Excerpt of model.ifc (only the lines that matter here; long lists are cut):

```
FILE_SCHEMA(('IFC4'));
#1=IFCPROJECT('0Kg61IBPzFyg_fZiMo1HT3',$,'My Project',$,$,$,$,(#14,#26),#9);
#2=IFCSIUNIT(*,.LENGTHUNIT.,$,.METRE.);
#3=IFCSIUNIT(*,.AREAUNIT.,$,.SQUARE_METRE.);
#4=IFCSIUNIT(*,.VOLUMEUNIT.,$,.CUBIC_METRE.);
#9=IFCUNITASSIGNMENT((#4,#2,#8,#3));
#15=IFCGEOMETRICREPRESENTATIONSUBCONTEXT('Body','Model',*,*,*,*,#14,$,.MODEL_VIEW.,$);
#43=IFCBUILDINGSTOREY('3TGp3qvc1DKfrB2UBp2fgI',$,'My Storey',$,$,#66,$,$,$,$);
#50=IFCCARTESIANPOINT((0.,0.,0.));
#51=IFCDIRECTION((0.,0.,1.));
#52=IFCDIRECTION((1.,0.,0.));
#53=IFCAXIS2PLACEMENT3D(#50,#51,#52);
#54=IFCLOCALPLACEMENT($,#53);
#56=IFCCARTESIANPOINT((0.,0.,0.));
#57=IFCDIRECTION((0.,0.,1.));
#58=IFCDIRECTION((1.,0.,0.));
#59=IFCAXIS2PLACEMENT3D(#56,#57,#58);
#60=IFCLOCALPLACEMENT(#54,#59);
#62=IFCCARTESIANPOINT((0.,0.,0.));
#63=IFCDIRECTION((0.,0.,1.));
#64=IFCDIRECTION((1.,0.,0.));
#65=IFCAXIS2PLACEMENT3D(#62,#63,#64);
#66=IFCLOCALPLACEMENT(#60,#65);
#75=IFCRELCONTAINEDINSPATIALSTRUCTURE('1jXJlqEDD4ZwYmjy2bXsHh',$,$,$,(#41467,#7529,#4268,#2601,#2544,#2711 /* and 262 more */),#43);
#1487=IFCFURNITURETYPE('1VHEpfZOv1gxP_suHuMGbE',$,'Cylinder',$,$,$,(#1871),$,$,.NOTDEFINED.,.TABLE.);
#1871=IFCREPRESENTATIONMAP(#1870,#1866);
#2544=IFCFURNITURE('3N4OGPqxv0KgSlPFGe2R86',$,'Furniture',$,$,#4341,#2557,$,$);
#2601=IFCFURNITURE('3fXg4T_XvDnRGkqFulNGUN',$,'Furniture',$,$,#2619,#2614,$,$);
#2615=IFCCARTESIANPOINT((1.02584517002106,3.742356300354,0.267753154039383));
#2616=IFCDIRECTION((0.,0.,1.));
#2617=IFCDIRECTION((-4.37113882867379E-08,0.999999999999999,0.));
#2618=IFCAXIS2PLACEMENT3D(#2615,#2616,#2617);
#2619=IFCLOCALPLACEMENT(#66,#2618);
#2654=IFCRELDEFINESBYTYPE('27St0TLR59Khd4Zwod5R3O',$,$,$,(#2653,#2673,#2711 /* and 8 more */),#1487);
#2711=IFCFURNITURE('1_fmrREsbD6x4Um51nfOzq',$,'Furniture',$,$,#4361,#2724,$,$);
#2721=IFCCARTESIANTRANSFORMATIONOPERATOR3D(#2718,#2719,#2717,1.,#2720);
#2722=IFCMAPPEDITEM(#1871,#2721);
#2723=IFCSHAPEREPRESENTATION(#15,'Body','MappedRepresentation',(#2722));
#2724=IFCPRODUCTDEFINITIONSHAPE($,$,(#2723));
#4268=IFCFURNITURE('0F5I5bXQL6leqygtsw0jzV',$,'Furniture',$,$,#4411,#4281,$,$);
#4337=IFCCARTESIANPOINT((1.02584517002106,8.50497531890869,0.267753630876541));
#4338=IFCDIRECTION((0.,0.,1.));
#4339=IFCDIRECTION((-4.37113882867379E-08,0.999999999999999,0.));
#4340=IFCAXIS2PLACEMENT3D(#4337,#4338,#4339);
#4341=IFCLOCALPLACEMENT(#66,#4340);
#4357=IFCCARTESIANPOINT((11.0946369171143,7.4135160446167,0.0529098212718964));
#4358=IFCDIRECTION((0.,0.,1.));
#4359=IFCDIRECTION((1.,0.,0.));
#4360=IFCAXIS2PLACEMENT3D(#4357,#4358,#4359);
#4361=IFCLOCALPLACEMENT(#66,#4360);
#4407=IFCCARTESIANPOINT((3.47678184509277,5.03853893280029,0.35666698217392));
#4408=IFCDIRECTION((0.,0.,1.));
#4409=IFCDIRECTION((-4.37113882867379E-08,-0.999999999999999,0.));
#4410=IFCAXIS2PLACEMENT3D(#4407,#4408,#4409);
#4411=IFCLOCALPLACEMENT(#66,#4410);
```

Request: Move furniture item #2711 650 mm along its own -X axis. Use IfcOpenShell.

```python
import ifcopenshell
import ifcopenshell.api.geometry
import ifcopenshell.util.placement
import ifcopenshell.util.unit

model = ifcopenshell.open("model.ifc")
unit_scale = ifcopenshell.util.unit.calculate_unit_scale(model)

item = model.by_guid("1_fmrREsbD6x4Um51nfOzq")
matrix = ifcopenshell.util.placement.get_local_placement(item.ObjectPlacement)
matrix[:3, 3] -= matrix[:3, 0] * 0.65 / unit_scale
ifcopenshell.api.geometry.edit_object_placement(model, product=item, matrix=matrix, is_si=False)

print(ifcopenshell.util.placement.get_local_placement(item.ObjectPlacement).round(3) + 0.0)

model.write("model-out.ifc")
```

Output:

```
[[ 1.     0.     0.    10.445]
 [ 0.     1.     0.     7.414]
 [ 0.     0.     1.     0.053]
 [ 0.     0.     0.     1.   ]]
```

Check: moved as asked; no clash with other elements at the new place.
